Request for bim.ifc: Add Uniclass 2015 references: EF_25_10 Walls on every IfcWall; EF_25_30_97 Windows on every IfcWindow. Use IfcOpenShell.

First a look at what the model holds.

```python
import ifcopenshell

model = ifcopenshell.open("bim.ifc")
print(model.schema)
print("classifications:", [c.Name for c in model.by_type("IfcClassification")])
for ifc_class in ("IfcDoor", "IfcRoof", "IfcStair", "IfcWall", "IfcWindow"):
    print(ifc_class, len(model.by_type(ifc_class)))
```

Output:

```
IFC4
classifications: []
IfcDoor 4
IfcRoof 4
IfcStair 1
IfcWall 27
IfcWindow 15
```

```python
import ifcopenshell
import ifcopenshell.api.classification

model = ifcopenshell.open("bim.ifc")

system = ifcopenshell.api.classification.add_classification(model, classification="Uniclass 2015")

codes = {
    "IfcWall": ("EF_25_10", "Walls"),
    "IfcWindow": ("EF_25_30_97", "Windows"),
}
for ifc_class, (code, name) in codes.items():
    products = model.by_type(ifc_class)
    ifcopenshell.api.classification.add_reference(
        model, products=products, classification=system, identification=code, name=name
    )
    print(code, len(products))

model.write("bim_v2.ifc")
```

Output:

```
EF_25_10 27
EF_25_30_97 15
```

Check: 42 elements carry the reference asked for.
